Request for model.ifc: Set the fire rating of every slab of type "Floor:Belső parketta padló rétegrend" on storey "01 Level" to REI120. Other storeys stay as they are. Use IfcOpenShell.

First a look at what the model holds.

```python
import ifcopenshell
import ifcopenshell.util.element

model = ifcopenshell.open("model.ifc")
print(model.schema)
storey = next(s for s in model.by_type("IfcBuildingStorey") if s.Name == "01 Level")
slabs = [e for e in ifcopenshell.util.element.get_decomposition(storey) if e.is_a("IfcSlab")]
seen = {}
for e in slabs:
    element_type = ifcopenshell.util.element.get_type(e)
    key = (element_type.Name if element_type != e and element_type else None, ifcopenshell.util.element.get_pset(e, "Pset_SlabCommon", "FireRating"))
    seen[key] = seen.get(key, 0) + 1
for (name, value), count in sorted(seen.items(), key=str):
    print(count, "x", name, "|", value)
```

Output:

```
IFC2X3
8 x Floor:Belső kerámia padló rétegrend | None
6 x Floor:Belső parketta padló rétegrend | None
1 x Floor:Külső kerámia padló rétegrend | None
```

```python
import ifcopenshell
import ifcopenshell.api.pset
import ifcopenshell.util.element

model = ifcopenshell.open("model.ifc")

storey = next(s for s in model.by_type("IfcBuildingStorey") if s.Name == "01 Level")
slabs = [e for e in ifcopenshell.util.element.get_decomposition(storey) if e.is_a("IfcSlab")]

count = 0
for e in slabs:
    element_type = ifcopenshell.util.element.get_type(e)
    if element_type in (None, e) or element_type.Name != "Floor:Belső parketta padló rétegrend":
        continue
    # add_pset returns the element's existing set when there is one.
    pset = ifcopenshell.api.pset.add_pset(model, product=e, name="Pset_SlabCommon")
    ifcopenshell.api.pset.edit_pset(model, pset=pset, properties={"FireRating": "REI120"})
    count += 1

print(count, "slabs updated")

model.write("model_rev.ifc")
```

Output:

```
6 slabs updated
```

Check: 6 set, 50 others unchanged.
